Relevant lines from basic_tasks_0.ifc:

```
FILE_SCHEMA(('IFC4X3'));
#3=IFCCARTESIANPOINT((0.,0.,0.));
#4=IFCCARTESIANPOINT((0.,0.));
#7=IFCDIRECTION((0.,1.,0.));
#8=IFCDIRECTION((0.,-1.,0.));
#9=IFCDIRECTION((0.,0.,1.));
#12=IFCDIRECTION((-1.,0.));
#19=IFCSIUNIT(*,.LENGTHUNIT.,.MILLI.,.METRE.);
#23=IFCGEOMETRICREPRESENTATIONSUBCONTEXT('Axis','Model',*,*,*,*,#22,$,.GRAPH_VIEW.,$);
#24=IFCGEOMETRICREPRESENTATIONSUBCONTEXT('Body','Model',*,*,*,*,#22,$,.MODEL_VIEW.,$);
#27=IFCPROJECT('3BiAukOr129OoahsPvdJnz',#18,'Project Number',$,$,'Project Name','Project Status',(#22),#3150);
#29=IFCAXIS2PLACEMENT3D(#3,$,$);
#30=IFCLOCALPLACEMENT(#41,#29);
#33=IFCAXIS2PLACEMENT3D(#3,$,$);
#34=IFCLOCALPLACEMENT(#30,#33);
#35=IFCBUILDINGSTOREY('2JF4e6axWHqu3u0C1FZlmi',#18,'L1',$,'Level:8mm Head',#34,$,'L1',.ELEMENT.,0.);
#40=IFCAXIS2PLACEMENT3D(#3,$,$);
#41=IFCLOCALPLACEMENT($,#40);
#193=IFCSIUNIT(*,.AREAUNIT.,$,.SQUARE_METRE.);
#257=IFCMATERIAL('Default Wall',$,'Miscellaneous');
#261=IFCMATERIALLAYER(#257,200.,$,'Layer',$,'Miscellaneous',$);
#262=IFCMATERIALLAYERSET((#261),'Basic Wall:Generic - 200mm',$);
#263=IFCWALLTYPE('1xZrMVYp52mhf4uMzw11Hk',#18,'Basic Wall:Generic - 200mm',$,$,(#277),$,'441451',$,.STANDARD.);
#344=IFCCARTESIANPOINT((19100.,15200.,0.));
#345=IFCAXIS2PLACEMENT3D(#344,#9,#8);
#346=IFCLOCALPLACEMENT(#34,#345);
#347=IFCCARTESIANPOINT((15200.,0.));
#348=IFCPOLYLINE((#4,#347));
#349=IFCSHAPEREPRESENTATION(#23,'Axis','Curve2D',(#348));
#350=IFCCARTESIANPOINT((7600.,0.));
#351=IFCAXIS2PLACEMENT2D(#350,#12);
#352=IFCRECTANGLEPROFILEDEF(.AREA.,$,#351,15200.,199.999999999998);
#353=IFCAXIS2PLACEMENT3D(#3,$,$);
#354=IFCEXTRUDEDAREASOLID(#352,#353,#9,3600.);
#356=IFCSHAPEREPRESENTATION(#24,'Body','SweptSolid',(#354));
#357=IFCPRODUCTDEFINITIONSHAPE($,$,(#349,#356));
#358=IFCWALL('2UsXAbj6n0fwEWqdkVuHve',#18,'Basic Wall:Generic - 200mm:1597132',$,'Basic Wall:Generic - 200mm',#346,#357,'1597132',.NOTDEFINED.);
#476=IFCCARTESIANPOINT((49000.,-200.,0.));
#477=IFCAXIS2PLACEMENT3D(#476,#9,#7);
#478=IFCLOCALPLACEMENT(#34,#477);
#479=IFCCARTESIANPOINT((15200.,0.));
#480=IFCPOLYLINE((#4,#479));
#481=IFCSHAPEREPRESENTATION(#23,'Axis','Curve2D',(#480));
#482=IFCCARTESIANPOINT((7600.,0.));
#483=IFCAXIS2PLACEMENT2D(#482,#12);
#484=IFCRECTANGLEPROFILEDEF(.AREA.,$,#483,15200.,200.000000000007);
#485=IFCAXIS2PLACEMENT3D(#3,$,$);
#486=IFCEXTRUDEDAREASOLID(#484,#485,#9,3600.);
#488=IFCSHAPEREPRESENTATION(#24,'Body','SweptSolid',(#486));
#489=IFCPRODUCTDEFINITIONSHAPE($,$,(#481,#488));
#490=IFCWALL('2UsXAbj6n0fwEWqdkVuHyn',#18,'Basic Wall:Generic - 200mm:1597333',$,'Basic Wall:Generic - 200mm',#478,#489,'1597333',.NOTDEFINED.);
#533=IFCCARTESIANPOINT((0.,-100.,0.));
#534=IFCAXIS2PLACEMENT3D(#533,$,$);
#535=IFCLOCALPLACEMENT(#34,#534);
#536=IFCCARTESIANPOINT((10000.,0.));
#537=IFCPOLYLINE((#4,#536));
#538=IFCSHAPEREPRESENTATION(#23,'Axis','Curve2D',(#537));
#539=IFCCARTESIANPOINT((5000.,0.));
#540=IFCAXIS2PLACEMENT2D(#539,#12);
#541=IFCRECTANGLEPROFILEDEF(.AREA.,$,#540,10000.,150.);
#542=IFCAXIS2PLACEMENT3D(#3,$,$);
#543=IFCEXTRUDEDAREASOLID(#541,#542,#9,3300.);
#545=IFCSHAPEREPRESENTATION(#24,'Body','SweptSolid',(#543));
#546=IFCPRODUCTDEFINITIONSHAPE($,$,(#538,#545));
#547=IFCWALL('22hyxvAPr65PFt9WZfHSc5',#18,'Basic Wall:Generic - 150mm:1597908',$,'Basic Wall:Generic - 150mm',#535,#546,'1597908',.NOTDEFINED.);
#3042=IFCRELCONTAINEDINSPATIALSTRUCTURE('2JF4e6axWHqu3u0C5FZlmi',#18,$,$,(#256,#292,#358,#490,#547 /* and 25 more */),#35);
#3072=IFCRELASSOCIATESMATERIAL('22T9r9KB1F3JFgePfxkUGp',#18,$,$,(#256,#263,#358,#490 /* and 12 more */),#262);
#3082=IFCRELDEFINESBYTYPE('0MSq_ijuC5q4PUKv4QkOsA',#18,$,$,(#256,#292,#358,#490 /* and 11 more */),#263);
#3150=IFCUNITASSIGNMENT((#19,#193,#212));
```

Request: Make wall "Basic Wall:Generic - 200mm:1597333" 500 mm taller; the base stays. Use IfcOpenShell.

```python
import ifcopenshell
import ifcopenshell.geom
import ifcopenshell.util.representation
import ifcopenshell.util.shape
import ifcopenshell.util.unit

model = ifcopenshell.open("basic_tasks_0.ifc")
unit_scale = ifcopenshell.util.unit.calculate_unit_scale(model)
settings = ifcopenshell.geom.settings()


def volume(element):
    """Net volume in cubic metres, openings subtracted."""
    shape = ifcopenshell.geom.create_shape(settings, element)
    return ifcopenshell.util.shape.get_volume(shape.geometry)


wall = model.by_guid("2UsXAbj6n0fwEWqdkVuHyn")
before = volume(wall)

body = ifcopenshell.util.representation.get_representation(wall, "Model", "Body")
solid = body.Items[0]
old_height = solid.Depth
solid.Depth += 0.5 / unit_scale
after = volume(wall)

print(f"height {old_height:g} -> {solid.Depth:g}, volume {before:.3f} -> {after:.3f} m3")

model.write("basic_tasks_0_edited.ifc")
```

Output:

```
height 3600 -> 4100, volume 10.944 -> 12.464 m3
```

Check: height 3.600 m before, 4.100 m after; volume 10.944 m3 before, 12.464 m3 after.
